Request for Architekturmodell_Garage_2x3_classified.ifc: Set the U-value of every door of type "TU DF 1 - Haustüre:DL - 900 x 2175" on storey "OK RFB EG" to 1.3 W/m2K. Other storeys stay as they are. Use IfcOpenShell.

First a look at what the model holds.

```python
import ifcopenshell
import ifcopenshell.util.element

model = ifcopenshell.open("Architekturmodell_Garage_2x3_classified.ifc")
print(model.schema)
storey = next(s for s in model.by_type("IfcBuildingStorey") if s.Name == "OK RFB EG")
doors = [e for e in ifcopenshell.util.element.get_decomposition(storey) if e.is_a("IfcDoor")]
seen = {}
for e in doors:
    element_type = ifcopenshell.util.element.get_type(e)
    key = (element_type.Name if element_type != e and element_type else None, ifcopenshell.util.element.get_pset(e, "Pset_DoorCommon", "ThermalTransmittance"))
    seen[key] = seen.get(key, 0) + 1
for (name, value), count in sorted(seen.items(), key=str):
    print(count, "x", name, "|", value)
```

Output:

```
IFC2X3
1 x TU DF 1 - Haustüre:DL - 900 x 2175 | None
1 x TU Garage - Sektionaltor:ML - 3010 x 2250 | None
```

```python
import ifcopenshell
import ifcopenshell.api.pset
import ifcopenshell.util.element

model = ifcopenshell.open("Architekturmodell_Garage_2x3_classified.ifc")

storey = next(s for s in model.by_type("IfcBuildingStorey") if s.Name == "OK RFB EG")
doors = [e for e in ifcopenshell.util.element.get_decomposition(storey) if e.is_a("IfcDoor")]

count = 0
for e in doors:
    element_type = ifcopenshell.util.element.get_type(e)
    if element_type in (None, e) or element_type.Name != "TU DF 1 - Haustüre:DL - 900 x 2175":
        continue
    # add_pset returns the element's existing set when there is one.
    pset = ifcopenshell.api.pset.add_pset(model, product=e, name="Pset_DoorCommon")
    ifcopenshell.api.pset.edit_pset(model, pset=pset, properties={"ThermalTransmittance": 1.3})
    count += 1

print(count, "doors updated")

model.write("Architekturmodell_Garage_2x3_classified_updated.ifc")
```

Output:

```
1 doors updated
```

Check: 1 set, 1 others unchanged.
